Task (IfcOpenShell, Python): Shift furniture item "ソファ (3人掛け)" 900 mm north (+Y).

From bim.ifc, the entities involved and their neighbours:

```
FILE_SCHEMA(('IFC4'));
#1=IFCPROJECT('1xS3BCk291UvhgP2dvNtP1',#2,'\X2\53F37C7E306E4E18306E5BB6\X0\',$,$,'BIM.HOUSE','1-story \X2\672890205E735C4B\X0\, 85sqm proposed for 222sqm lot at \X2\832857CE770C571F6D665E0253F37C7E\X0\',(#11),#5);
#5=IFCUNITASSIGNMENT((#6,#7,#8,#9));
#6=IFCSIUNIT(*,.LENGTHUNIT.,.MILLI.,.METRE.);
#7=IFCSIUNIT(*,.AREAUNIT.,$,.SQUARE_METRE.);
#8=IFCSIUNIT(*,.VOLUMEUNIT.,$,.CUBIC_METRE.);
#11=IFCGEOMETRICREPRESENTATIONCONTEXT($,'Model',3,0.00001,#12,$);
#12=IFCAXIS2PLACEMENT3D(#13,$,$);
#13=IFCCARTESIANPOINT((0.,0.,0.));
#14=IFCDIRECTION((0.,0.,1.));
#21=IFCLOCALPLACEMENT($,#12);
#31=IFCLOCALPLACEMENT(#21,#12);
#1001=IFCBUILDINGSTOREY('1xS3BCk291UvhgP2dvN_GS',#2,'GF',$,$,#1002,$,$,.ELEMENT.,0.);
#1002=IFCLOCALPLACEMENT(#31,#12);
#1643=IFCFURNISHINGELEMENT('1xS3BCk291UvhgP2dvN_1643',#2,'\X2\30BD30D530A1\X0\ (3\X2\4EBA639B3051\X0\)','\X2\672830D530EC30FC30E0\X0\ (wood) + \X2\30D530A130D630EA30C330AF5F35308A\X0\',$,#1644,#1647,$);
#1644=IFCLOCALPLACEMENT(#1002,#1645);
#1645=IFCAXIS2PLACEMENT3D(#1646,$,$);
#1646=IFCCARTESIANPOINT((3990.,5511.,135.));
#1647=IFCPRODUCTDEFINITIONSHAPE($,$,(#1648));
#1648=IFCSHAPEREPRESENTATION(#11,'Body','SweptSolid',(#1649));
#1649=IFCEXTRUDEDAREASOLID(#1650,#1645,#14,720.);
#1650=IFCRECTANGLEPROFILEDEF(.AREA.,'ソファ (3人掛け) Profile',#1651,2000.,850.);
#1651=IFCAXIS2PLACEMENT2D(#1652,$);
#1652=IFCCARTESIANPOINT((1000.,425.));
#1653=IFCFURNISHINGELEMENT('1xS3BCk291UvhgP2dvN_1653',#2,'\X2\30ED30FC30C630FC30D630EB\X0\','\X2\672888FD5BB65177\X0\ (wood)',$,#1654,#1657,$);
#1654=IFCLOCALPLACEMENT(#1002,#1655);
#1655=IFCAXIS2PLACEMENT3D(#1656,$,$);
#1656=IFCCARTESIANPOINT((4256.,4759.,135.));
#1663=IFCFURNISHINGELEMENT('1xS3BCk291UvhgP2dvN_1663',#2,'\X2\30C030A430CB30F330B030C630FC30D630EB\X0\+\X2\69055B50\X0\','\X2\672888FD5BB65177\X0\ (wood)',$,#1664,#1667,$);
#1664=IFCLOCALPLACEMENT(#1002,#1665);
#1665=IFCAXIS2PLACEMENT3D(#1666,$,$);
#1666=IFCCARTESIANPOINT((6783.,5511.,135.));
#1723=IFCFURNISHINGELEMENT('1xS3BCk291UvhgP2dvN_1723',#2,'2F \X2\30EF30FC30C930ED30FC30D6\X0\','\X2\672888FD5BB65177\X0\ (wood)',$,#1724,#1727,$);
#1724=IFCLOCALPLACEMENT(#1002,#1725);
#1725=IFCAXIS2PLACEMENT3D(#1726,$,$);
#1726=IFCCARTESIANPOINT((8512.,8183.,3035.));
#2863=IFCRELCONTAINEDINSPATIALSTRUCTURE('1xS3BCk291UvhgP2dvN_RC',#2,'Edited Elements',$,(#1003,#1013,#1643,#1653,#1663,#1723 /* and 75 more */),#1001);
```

```python
import ifcopenshell
import ifcopenshell.api.geometry
import ifcopenshell.util.placement
import ifcopenshell.util.unit

model = ifcopenshell.open("bim.ifc")
unit_scale = ifcopenshell.util.unit.calculate_unit_scale(model)

item = model.by_guid("1xS3BCk291UvhgP2dvN_1643")
matrix = ifcopenshell.util.placement.get_local_placement(item.ObjectPlacement)
matrix[1, 3] += 0.9 / unit_scale
ifcopenshell.api.geometry.edit_object_placement(model, product=item, matrix=matrix, is_si=False)

print(ifcopenshell.util.placement.get_local_placement(item.ObjectPlacement).round(3) + 0.0)

model.write("bim_updated.ifc")
```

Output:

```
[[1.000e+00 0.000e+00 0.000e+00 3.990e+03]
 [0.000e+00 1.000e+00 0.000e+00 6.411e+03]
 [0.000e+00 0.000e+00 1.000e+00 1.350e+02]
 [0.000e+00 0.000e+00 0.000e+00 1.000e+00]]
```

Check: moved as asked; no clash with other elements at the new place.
